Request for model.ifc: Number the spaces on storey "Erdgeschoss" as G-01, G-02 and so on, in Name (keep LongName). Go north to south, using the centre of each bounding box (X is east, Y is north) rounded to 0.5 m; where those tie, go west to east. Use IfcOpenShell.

First a look at what the model holds.

```python
import ifcopenshell
import ifcopenshell.util.element
import ifcopenshell.util.placement

model = ifcopenshell.open("model.ifc")
print(model.schema)
storey = next(s for s in model.by_type("IfcBuildingStorey") if s.Name == "Erdgeschoss")
spaces = [e for e in ifcopenshell.util.element.get_decomposition(storey) if e.is_a("IfcSpace")]
for e in sorted(spaces, key=lambda e: e.id()):
    origin = ifcopenshell.util.placement.get_local_placement(e.ObjectPlacement)[:3, 3]
    print(e.id(), e.Name, e.LongName, origin.round(2) + 0.0, sep=" | ")
```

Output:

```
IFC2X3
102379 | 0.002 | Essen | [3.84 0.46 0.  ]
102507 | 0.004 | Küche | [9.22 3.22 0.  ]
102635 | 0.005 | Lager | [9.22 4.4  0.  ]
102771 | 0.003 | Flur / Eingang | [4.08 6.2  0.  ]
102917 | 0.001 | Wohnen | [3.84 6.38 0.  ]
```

```python
import ifcopenshell
import ifcopenshell.geom
import ifcopenshell.util.element
import ifcopenshell.util.shape

model = ifcopenshell.open("model.ifc")
settings = ifcopenshell.geom.settings()
settings.set("use-world-coords", True)


def centre(element):
    shape = ifcopenshell.geom.create_shape(settings, element)
    return ifcopenshell.util.shape.get_bbox_centroid(shape.geometry)


storey = next(s for s in model.by_type("IfcBuildingStorey") if s.Name == "Erdgeschoss")
spaces = [e for e in ifcopenshell.util.element.get_decomposition(storey) if e.is_a("IfcSpace")]

# Insertion points can sit at a corner or the storey origin, so sort by the geometry (in metres).
centres = {e: centre(e) for e in spaces}
spaces.sort(key=lambda e: (-round(centres[e][1] / 0.5), centres[e][0]))

for i, e in enumerate(spaces, start=1):
    number = f"G-{i:02d}"
    e.Name = number
    print(e.id(), number)

model.write("model_v2.ifc")
```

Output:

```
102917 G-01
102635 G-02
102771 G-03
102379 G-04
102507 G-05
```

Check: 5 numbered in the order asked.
